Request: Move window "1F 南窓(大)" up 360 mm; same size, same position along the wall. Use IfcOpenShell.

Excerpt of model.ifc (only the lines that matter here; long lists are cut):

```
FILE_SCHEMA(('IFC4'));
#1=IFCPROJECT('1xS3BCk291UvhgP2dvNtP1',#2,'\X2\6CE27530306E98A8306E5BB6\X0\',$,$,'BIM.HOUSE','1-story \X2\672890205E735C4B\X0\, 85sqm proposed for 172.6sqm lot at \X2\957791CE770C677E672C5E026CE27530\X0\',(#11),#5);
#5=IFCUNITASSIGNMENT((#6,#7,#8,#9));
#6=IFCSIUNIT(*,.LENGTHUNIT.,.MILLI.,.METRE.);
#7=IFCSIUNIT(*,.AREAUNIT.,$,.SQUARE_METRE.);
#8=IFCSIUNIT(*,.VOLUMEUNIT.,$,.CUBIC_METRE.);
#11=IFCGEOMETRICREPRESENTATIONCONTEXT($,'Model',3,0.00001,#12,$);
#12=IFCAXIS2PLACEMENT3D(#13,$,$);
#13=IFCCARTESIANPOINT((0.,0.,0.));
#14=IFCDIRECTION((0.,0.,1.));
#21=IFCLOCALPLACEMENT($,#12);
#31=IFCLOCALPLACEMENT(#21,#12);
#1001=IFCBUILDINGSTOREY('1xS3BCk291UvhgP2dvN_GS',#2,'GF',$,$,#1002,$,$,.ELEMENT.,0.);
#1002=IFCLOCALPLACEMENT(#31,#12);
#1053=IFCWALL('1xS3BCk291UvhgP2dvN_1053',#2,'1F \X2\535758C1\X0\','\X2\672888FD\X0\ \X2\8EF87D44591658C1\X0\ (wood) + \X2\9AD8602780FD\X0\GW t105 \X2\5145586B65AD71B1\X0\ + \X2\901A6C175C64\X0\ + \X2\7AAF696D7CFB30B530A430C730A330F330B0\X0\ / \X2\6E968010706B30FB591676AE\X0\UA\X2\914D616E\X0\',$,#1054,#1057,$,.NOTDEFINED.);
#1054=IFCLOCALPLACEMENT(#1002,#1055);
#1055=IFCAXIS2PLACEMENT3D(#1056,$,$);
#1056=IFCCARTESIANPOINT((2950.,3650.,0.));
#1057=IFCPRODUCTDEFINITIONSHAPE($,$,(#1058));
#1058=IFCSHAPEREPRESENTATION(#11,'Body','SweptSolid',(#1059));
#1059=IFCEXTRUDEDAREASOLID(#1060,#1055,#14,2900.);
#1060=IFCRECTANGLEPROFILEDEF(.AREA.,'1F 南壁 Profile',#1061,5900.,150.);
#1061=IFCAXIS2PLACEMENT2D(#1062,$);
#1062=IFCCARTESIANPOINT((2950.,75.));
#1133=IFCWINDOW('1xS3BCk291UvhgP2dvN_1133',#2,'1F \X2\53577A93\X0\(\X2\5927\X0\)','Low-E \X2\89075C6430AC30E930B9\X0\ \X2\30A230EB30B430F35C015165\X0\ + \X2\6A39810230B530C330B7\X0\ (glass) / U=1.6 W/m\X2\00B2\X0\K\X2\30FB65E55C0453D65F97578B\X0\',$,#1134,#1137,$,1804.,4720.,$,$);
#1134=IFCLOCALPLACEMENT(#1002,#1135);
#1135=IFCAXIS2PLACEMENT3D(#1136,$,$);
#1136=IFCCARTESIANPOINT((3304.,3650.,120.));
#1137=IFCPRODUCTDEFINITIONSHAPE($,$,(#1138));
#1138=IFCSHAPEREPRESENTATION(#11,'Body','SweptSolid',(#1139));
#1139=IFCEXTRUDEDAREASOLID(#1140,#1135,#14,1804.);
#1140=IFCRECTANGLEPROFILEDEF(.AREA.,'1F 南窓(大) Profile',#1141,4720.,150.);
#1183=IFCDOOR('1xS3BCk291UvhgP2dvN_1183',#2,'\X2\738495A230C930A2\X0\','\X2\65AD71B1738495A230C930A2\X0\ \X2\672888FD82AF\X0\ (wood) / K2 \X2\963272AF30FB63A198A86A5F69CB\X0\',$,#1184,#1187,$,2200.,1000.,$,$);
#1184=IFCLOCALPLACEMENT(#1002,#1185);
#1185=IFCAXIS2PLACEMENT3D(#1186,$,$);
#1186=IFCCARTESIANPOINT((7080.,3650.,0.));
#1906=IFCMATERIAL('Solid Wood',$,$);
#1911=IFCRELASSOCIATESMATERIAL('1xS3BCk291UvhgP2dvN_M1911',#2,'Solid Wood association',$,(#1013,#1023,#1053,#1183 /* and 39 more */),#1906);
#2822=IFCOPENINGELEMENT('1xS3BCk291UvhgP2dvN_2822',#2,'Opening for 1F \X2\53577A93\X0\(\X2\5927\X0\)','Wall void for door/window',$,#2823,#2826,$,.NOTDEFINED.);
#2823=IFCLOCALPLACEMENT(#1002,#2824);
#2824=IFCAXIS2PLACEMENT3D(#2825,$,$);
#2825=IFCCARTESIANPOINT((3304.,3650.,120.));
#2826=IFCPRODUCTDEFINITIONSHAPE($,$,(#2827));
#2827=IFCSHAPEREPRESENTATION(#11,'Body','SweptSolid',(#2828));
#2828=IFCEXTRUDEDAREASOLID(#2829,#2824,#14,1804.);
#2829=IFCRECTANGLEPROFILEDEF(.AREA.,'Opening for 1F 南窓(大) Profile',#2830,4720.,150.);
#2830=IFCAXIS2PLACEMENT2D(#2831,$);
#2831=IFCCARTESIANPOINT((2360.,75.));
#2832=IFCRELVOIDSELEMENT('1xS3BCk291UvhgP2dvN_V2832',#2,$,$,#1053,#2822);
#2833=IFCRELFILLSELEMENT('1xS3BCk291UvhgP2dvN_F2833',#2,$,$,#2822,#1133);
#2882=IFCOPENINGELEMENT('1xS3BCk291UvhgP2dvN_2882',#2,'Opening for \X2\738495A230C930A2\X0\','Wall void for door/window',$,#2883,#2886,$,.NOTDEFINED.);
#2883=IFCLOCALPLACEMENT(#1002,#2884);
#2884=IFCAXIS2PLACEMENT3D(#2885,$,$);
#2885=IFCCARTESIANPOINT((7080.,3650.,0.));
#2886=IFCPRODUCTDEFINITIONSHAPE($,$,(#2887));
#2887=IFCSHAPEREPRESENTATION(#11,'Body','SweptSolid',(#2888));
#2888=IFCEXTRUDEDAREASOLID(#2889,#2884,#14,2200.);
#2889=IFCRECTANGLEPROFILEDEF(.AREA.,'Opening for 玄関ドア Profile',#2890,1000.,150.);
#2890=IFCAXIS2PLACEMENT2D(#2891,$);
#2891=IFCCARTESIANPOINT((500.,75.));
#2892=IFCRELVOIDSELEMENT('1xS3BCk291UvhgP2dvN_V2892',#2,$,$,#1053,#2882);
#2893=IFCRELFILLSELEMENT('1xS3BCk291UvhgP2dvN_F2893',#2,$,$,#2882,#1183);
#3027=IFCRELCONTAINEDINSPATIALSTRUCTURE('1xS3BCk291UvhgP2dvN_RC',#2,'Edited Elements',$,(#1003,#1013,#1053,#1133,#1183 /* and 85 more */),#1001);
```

```python
import numpy as np
import ifcopenshell
import ifcopenshell.api.geometry
import ifcopenshell.util.placement
import ifcopenshell.util.unit

model = ifcopenshell.open("model.ifc")
unit_scale = ifcopenshell.util.unit.calculate_unit_scale(model)

window = model.by_id(1133)
opening = window.FillsVoids[0].RelatingOpeningElement
dz = 360.0

shift = np.array([0.0, 0.0, dz])
# The window is not placed relative to its opening, so move both.
for product in (opening, window):
    matrix = ifcopenshell.util.placement.get_local_placement(product.ObjectPlacement)
    matrix[:3, 3] += shift
    ifcopenshell.api.geometry.edit_object_placement(model, product=product, matrix=matrix, is_si=False)

print(f"moved by {dz * unit_scale:+.3f} m")

model.write("model_updated.ifc")
```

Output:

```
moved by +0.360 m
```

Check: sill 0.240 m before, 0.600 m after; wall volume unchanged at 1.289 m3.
